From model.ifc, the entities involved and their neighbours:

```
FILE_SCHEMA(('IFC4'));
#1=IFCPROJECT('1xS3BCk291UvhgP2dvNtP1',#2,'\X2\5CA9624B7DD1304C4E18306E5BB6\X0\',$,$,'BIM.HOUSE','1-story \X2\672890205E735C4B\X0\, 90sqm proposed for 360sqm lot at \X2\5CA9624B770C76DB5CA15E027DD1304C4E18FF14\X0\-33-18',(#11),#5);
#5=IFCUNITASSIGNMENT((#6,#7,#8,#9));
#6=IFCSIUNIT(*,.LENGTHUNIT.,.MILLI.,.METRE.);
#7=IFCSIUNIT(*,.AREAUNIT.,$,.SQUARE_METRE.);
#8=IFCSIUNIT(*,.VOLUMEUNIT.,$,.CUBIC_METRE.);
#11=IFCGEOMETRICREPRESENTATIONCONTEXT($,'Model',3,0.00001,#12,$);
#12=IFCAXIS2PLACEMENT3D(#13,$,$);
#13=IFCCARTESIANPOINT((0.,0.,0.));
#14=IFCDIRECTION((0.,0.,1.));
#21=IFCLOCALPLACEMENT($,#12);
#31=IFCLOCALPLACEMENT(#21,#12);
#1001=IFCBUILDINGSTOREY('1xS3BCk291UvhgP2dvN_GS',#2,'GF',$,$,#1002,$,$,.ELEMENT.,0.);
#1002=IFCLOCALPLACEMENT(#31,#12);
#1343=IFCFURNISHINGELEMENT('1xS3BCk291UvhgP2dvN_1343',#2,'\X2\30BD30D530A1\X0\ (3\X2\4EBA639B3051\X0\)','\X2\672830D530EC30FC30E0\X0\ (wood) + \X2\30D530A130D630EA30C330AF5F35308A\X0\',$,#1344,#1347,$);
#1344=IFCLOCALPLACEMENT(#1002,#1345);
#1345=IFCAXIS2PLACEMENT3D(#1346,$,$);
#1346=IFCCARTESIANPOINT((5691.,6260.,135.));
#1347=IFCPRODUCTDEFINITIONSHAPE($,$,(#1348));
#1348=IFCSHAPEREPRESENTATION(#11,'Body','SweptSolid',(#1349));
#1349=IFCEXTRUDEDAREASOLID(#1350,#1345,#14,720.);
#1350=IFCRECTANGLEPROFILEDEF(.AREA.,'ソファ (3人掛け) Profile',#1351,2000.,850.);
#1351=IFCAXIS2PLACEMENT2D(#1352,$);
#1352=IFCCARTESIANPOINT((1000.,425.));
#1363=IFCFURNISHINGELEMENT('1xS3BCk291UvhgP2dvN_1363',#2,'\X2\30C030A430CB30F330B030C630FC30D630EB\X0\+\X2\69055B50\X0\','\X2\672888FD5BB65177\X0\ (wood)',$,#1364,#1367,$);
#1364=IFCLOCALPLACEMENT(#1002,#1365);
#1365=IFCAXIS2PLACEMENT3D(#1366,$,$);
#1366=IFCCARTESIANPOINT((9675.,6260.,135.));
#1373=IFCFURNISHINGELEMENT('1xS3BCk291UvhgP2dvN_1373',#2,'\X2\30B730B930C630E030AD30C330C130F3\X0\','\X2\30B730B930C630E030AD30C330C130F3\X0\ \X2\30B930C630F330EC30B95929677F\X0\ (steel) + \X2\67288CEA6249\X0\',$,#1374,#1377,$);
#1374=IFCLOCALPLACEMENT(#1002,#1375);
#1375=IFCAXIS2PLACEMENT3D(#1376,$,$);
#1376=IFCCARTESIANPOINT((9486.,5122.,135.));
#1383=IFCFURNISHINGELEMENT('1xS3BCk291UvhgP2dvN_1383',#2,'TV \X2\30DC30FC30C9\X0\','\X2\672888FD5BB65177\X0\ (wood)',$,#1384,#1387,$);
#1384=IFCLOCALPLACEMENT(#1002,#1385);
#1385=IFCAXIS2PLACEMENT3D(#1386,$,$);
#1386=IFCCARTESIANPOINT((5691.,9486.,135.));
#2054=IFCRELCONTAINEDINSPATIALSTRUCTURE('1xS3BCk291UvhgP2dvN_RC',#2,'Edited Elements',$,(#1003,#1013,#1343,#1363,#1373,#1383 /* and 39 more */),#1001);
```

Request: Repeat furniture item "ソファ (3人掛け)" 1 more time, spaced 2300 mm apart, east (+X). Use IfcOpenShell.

```python
import numpy as np
import ifcopenshell
import ifcopenshell.api.geometry
import ifcopenshell.api.root
import ifcopenshell.util.element
import ifcopenshell.util.placement
import ifcopenshell.util.unit

model = ifcopenshell.open("model.ifc")
unit_scale = ifcopenshell.util.unit.calculate_unit_scale(model)


def reuse_history(source, copy):
    """copy_class also copies each property set's owner history, people and application; keep the originals."""
    for rel in copy.IsDefinedBy:
        if rel.is_a("IfcRelDefinesByProperties") and (history := rel.RelatingPropertyDefinition.OwnerHistory):
            rel.RelatingPropertyDefinition.OwnerHistory = source.OwnerHistory
            ifcopenshell.util.element.remove_deep2(model, history)


source = model.by_guid("1xS3BCk291UvhgP2dvN_1343")
base = ifcopenshell.util.placement.get_local_placement(source.ObjectPlacement)
step = np.array([1.0, 0.0, 0.0]) * 2.3 / unit_scale

for i in range(1, 2):
    copy = ifcopenshell.api.root.copy_class(model, product=source)
    copy.Representation = ifcopenshell.util.element.copy_deep(
        model, source.Representation, exclude=["IfcGeometricRepresentationContext", "IfcRepresentationMap"]
    )
    reuse_history(source, copy)
    matrix = base.copy()
    matrix[:3, 3] += i * step
    print("added at", matrix[:3, 3].round(3) + 0.0)
    ifcopenshell.api.geometry.edit_object_placement(model, product=copy, matrix=matrix, is_si=False)

model.write("model_v2.ifc")
```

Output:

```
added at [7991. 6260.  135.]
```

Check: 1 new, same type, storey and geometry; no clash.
